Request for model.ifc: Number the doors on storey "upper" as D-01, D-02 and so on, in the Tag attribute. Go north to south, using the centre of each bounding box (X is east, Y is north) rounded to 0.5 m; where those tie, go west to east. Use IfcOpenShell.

First a look at what the model holds.

```python
import ifcopenshell
import ifcopenshell.util.element
import ifcopenshell.util.placement

model = ifcopenshell.open("model.ifc")
print(model.schema)
storey = next(s for s in model.by_type("IfcBuildingStorey") if s.Name == "upper")
doors = [e for e in ifcopenshell.util.element.get_decomposition(storey) if e.is_a("IfcDoor")]
for e in sorted(doors, key=lambda e: e.id()):
    origin = ifcopenshell.util.placement.get_local_placement(e.ObjectPlacement)[:3, 3]
    print(e.id(), e.Tag, e.Name, origin.round(2) + 0.0, sep=" | ")
```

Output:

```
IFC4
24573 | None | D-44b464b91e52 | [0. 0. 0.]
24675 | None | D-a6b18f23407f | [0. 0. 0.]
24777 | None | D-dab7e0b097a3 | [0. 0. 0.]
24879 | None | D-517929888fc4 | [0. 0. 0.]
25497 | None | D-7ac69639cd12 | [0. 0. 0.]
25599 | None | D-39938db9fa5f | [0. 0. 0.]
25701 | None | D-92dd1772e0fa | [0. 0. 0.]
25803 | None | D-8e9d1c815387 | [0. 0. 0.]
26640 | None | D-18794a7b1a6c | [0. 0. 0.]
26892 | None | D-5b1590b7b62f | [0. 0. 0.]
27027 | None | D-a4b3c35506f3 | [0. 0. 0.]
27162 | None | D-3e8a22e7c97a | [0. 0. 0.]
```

```python
import ifcopenshell
import ifcopenshell.geom
import ifcopenshell.util.element
import ifcopenshell.util.shape

model = ifcopenshell.open("model.ifc")
settings = ifcopenshell.geom.settings()
settings.set("use-world-coords", True)


def centre(element):
    shape = ifcopenshell.geom.create_shape(settings, element)
    return ifcopenshell.util.shape.get_bbox_centroid(shape.geometry)


storey = next(s for s in model.by_type("IfcBuildingStorey") if s.Name == "upper")
doors = [e for e in ifcopenshell.util.element.get_decomposition(storey) if e.is_a("IfcDoor")]

# Insertion points can sit at a corner or the storey origin, so sort by the geometry (in metres).
centres = {e: centre(e) for e in doors}
doors.sort(key=lambda e: (-round(centres[e][1] / 0.5), centres[e][0]))

for i, e in enumerate(doors, start=1):
    number = f"D-{i:02d}"
    e.Tag = number
    print(e.id(), number)

model.write("model_v2.ifc")
```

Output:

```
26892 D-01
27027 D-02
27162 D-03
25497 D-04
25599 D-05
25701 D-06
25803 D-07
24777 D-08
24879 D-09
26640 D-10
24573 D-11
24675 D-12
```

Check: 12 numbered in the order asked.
